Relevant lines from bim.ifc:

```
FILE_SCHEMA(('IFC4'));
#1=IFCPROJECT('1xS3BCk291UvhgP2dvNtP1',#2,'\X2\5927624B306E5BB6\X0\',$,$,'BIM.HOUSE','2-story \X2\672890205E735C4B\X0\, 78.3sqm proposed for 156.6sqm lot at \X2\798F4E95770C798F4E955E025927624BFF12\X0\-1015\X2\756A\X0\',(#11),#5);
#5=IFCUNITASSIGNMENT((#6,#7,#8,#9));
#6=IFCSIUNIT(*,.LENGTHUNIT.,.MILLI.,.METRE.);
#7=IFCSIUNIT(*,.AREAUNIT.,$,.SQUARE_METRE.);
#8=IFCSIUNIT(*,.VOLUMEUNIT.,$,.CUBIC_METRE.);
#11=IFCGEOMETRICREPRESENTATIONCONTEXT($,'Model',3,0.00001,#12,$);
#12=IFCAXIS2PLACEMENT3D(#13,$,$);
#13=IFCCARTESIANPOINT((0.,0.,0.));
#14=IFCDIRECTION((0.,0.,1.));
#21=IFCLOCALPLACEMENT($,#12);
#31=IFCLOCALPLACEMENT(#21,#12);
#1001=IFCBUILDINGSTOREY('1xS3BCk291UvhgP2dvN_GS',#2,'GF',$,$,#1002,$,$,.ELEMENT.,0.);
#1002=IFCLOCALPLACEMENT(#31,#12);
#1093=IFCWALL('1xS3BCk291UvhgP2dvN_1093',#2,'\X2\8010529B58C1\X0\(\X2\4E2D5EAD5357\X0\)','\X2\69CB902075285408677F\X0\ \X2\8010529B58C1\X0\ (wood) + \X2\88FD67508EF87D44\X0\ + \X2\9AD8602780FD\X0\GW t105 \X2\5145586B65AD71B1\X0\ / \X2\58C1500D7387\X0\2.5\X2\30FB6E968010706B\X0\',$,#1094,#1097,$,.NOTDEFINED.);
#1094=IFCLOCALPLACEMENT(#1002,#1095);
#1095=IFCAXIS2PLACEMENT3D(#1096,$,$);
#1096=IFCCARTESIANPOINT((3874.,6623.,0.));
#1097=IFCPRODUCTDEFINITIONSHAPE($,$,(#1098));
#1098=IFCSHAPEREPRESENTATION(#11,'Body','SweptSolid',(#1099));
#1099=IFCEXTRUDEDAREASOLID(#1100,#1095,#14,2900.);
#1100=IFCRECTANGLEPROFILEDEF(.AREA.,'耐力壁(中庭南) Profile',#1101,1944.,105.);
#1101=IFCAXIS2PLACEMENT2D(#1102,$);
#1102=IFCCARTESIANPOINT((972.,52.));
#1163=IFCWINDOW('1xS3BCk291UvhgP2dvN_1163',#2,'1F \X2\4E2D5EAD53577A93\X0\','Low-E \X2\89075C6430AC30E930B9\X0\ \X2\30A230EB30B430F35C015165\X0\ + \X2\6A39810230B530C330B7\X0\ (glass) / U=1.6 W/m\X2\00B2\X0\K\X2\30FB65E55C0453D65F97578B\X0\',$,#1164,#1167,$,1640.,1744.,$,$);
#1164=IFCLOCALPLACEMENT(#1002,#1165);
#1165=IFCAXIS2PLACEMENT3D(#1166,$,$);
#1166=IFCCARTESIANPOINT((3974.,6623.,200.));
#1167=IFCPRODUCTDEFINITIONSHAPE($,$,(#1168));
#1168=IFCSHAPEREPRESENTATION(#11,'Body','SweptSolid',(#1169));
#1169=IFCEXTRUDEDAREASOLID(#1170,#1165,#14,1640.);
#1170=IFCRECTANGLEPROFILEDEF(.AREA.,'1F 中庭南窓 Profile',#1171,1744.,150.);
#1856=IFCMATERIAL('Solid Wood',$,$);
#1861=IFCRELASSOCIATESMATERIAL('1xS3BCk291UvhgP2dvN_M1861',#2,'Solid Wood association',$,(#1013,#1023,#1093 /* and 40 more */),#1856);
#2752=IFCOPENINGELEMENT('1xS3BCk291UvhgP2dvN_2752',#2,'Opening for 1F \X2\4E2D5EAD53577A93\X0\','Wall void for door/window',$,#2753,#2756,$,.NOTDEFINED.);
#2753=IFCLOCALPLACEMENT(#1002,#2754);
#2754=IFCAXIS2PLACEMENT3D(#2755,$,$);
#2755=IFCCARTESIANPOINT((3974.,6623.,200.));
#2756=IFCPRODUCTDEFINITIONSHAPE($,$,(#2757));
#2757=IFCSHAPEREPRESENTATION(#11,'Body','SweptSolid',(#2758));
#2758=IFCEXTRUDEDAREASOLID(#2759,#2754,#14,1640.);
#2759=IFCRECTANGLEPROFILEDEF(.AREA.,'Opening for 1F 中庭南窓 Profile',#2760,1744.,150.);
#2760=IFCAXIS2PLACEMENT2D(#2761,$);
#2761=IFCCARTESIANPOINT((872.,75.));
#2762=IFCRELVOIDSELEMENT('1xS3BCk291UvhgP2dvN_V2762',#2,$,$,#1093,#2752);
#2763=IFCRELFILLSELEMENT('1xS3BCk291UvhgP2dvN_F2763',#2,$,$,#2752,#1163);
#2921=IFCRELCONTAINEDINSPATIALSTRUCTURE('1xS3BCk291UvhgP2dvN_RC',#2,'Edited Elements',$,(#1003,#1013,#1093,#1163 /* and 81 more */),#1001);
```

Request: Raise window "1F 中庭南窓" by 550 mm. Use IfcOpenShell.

```python
import numpy as np
import ifcopenshell
import ifcopenshell.api.geometry
import ifcopenshell.util.placement
import ifcopenshell.util.unit

model = ifcopenshell.open("bim.ifc")
unit_scale = ifcopenshell.util.unit.calculate_unit_scale(model)

window = model.by_id(1163)
opening = window.FillsVoids[0].RelatingOpeningElement
dz = 0.55 / unit_scale

shift = np.array([0.0, 0.0, dz])
# The window is not placed relative to its opening, so move both.
for product in (opening, window):
    matrix = ifcopenshell.util.placement.get_local_placement(product.ObjectPlacement)
    matrix[:3, 3] += shift
    ifcopenshell.api.geometry.edit_object_placement(model, product=product, matrix=matrix, is_si=False)

print(f"moved by {dz * unit_scale:+.3f} m")

model.write("bim-out.ifc")
```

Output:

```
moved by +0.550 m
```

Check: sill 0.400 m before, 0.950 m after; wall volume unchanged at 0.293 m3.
